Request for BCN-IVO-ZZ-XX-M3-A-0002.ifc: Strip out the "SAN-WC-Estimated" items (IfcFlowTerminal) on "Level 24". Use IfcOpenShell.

First a look at what the model holds.

```python
import ifcopenshell
import ifcopenshell.util.element

model = ifcopenshell.open("BCN-IVO-ZZ-XX-M3-A-0002.ifc")
print(model.schema)
storey = next(s for s in model.by_type("IfcBuildingStorey") if s.Name == "Level 24")
terminals = [e for e in ifcopenshell.util.element.get_decomposition(storey) if e.is_a("IfcFlowTerminal")]
seen = {}
for e in terminals:
    element_type = ifcopenshell.util.element.get_type(e)
    name = element_type.Name if element_type not in (None, e) else None
    seen[name] = seen.get(name, 0) + 1
for name, count in sorted(seen.items(), key=str):
    print(count, "x", name)
```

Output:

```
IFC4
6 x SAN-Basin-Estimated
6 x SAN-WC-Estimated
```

```python
import ifcopenshell
import ifcopenshell.api.root
import ifcopenshell.util.element

model = ifcopenshell.open("BCN-IVO-ZZ-XX-M3-A-0002.ifc")

storey = next(s for s in model.by_type("IfcBuildingStorey") if s.Name == "Level 24")
terminals = [e for e in ifcopenshell.util.element.get_decomposition(storey) if e.is_a("IfcFlowTerminal")]
targets = [e for e in terminals if (t := ifcopenshell.util.element.get_type(e)) not in (None, e) and t.Name == "SAN-WC-Estimated"]

for e in targets:
    ifcopenshell.api.root.remove_product(model, product=e)
print(len(targets), "removed")

model.write("BCN-IVO-ZZ-XX-M3-A-0002-out.ifc")
```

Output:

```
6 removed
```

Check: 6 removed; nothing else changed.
